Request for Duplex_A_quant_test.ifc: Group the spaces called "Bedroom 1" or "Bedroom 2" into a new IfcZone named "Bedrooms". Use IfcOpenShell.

First a look at what the model holds.

```python
import ifcopenshell

model = ifcopenshell.open("Duplex_A_quant_test.ifc")
print(model.schema)
seen = {}
for space in model.by_type("IfcSpace"):
    seen[space.LongName] = seen.get(space.LongName, 0) + 1
for name, count in sorted(seen.items(), key=str):
    print(count, "x", name)
print("zones:", [z.Name for z in model.by_type("IfcZone")][:20])
```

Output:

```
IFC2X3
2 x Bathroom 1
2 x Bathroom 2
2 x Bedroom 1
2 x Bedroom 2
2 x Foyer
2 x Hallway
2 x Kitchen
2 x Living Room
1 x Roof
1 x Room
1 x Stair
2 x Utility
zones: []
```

```python
import ifcopenshell
import ifcopenshell.api.group
import ifcopenshell.api.root

model = ifcopenshell.open("Duplex_A_quant_test.ifc")

names = {"Bedroom 1", "Bedroom 2"}
spaces = [s for s in model.by_type("IfcSpace") if s.LongName in names]

zone = ifcopenshell.api.root.create_entity(model, ifc_class="IfcZone", name="Bedrooms")
ifcopenshell.api.group.assign_group(model, products=spaces, group=zone)
print(len(spaces), "spaces in", zone.Name)

model.write("Duplex_A_quant_test_edited.ifc")
```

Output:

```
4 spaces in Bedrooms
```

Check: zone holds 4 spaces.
